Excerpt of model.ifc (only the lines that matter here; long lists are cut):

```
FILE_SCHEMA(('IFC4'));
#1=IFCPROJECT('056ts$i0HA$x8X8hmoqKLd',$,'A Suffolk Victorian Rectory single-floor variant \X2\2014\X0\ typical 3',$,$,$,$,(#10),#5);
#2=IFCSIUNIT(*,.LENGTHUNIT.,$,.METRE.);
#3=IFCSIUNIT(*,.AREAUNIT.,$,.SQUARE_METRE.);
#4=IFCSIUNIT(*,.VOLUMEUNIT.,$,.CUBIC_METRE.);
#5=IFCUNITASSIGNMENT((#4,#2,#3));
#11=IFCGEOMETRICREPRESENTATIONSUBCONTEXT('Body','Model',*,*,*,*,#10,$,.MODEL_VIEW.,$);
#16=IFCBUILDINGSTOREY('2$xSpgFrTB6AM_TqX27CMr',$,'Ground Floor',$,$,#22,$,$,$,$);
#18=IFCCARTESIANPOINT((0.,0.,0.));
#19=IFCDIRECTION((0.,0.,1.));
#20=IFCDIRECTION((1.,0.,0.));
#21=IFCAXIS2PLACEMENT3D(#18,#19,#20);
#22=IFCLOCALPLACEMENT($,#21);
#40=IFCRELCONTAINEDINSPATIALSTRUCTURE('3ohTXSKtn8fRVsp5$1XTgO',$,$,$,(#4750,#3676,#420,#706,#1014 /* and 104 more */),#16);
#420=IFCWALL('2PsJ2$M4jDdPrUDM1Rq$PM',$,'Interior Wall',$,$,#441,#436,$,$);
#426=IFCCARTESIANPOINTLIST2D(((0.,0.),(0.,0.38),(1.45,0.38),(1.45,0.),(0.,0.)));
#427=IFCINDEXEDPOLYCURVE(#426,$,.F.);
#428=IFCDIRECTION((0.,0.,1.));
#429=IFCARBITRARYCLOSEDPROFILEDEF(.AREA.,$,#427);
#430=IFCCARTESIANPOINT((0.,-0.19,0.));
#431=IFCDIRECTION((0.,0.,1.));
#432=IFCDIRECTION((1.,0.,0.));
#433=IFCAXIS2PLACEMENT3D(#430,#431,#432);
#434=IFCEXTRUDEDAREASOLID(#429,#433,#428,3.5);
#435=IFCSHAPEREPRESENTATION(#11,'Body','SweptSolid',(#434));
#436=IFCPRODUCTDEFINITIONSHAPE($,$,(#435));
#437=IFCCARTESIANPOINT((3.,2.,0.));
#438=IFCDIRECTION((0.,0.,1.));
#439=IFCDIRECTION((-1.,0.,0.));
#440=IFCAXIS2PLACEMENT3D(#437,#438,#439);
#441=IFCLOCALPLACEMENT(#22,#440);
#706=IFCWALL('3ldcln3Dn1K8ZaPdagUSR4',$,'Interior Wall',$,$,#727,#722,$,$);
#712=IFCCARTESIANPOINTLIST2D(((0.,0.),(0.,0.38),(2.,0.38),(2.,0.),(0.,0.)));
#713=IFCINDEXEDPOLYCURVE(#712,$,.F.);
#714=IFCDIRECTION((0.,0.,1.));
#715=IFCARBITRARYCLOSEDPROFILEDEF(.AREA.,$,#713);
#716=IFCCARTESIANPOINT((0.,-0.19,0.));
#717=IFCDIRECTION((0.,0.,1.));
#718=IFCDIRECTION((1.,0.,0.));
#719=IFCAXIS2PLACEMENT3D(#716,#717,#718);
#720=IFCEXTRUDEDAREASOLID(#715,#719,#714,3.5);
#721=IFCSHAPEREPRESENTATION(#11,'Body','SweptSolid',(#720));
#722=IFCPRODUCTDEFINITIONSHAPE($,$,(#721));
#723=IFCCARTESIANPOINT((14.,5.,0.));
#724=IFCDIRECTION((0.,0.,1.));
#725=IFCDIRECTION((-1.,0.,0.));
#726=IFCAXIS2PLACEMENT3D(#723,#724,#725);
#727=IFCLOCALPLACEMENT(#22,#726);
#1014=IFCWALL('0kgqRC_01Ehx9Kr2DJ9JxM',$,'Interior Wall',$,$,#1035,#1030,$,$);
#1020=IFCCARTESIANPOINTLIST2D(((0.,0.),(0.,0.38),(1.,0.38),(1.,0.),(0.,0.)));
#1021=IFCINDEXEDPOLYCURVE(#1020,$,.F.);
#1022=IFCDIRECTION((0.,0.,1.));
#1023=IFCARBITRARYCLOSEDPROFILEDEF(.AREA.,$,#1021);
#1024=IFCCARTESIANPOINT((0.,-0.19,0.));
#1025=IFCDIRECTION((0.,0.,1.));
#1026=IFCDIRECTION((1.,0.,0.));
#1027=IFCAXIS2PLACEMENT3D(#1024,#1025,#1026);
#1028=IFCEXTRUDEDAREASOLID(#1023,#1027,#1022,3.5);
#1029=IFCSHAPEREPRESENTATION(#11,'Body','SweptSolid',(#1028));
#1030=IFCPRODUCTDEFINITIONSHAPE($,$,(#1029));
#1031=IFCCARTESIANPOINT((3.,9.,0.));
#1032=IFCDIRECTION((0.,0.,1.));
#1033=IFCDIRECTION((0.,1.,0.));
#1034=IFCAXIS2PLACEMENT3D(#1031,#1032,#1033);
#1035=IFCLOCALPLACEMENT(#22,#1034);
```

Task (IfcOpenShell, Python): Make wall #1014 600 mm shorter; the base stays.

```python
import ifcopenshell
import ifcopenshell.geom
import ifcopenshell.util.representation
import ifcopenshell.util.shape
import ifcopenshell.util.unit

model = ifcopenshell.open("model.ifc")
unit_scale = ifcopenshell.util.unit.calculate_unit_scale(model)
settings = ifcopenshell.geom.settings()


def volume(element):
    """Net volume in cubic metres, openings subtracted."""
    shape = ifcopenshell.geom.create_shape(settings, element)
    return ifcopenshell.util.shape.get_volume(shape.geometry)


wall = model.by_guid("0kgqRC_01Ehx9Kr2DJ9JxM")
before = volume(wall)

body = ifcopenshell.util.representation.get_representation(wall, "Model", "Body")
solid = body.Items[0]
old_height = solid.Depth
solid.Depth -= 0.6 / unit_scale
after = volume(wall)

print(f"height {old_height:g} -> {solid.Depth:g}, volume {before:.3f} -> {after:.3f} m3")

model.write("model-out.ifc")
```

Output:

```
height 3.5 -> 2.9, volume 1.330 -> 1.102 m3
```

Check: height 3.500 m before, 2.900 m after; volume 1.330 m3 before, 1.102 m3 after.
